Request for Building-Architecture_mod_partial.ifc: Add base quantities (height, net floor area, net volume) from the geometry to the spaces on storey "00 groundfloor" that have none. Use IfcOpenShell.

First a look at what the model holds.

```python
import ifcopenshell
import ifcopenshell.util.element
import ifcopenshell.util.unit

model = ifcopenshell.open("Building-Architecture_mod_partial.ifc")
print(model.schema)
for unit_type in ("LENGTHUNIT", "AREAUNIT", "VOLUMEUNIT"):
    print(unit_type, ifcopenshell.util.unit.calculate_unit_scale(model, unit_type))
storey = next(s for s in model.by_type("IfcBuildingStorey") if s.Name == "00 groundfloor")
spaces = [e for e in ifcopenshell.util.element.get_decomposition(storey) if e.is_a("IfcSpace")]
for e in sorted(spaces, key=lambda e: e.id()):
    print(e.id(), e.is_a(), e.Name, list(ifcopenshell.util.element.get_psets(e, qtos_only=True)), sep=" | ")
```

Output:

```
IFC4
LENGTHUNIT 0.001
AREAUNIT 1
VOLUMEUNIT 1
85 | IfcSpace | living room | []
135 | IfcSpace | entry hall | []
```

```python
import ifcopenshell
import ifcopenshell.api.pset
import ifcopenshell.geom
import ifcopenshell.util.element
import ifcopenshell.util.shape
import ifcopenshell.util.unit

model = ifcopenshell.open("Building-Architecture_mod_partial.ifc")
unit_scale = ifcopenshell.util.unit.calculate_unit_scale(model)
area_scale = ifcopenshell.util.unit.calculate_unit_scale(model, "AREAUNIT")
volume_scale = ifcopenshell.util.unit.calculate_unit_scale(model, "VOLUMEUNIT")
settings = ifcopenshell.geom.settings()

storey = next(s for s in model.by_type("IfcBuildingStorey") if s.Name == "00 groundfloor")
spaces = [e for e in ifcopenshell.util.element.get_decomposition(storey) if e.is_a("IfcSpace")]

for e in sorted(spaces, key=lambda e: e.id()):
    if ifcopenshell.util.element.get_psets(e, qtos_only=True, should_inherit=False):
        continue
    # Geometry comes back in metres, in the element's own axes.
    shape = ifcopenshell.geom.create_shape(settings, e)
    values = {
        "Height": ifcopenshell.util.shape.get_z(shape.geometry) / unit_scale,
        "NetFloorArea": ifcopenshell.util.shape.get_footprint_area(shape.geometry) / area_scale,
        "NetVolume": ifcopenshell.util.shape.get_volume(shape.geometry) / volume_scale,
    }
    qto = ifcopenshell.api.pset.add_qto(model, product=e, name="Qto_SpaceBaseQuantities")
    ifcopenshell.api.pset.edit_qto(model, qto=qto, properties=values)
    print(e.id(), {k: round(v, 3) for k, v in values.items()})

model.write("Building-Architecture_mod_partial-out.ifc")
```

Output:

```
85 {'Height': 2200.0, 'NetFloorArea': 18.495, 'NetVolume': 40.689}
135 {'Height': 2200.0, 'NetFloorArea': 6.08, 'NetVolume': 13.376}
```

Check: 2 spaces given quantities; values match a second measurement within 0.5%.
